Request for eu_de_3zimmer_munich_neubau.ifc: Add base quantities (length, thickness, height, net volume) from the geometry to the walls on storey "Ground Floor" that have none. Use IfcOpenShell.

First a look at what the model holds.

```python
import ifcopenshell
import ifcopenshell.util.element
import ifcopenshell.util.unit

model = ifcopenshell.open("eu_de_3zimmer_munich_neubau.ifc")
print(model.schema)
for unit_type in ("LENGTHUNIT", "AREAUNIT", "VOLUMEUNIT"):
    print(unit_type, ifcopenshell.util.unit.calculate_unit_scale(model, unit_type))
storey = next(s for s in model.by_type("IfcBuildingStorey") if s.Name == "Ground Floor")
walls = [e for e in ifcopenshell.util.element.get_decomposition(storey) if e.is_a("IfcWall")]
for e in sorted(walls, key=lambda e: e.id()):
    print(e.id(), e.is_a(), e.Name, list(ifcopenshell.util.element.get_psets(e, qtos_only=True)), sep=" | ")
```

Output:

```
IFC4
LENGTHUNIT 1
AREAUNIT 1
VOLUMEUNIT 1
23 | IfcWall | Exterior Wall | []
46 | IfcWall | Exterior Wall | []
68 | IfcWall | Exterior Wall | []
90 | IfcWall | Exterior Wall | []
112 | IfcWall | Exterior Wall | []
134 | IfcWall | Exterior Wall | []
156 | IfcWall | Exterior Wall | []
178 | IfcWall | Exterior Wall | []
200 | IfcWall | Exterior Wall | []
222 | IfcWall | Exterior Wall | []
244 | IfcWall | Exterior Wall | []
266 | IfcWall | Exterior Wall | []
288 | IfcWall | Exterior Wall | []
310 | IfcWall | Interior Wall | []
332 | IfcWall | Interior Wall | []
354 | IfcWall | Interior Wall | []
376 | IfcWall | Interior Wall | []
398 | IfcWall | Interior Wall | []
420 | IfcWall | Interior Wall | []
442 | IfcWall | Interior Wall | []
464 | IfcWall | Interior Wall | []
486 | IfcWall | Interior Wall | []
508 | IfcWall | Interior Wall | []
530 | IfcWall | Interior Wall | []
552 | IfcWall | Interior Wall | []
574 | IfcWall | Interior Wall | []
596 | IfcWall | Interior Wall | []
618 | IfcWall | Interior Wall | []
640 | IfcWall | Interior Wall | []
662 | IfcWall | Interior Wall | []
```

```python
import ifcopenshell
import ifcopenshell.api.pset
import ifcopenshell.geom
import ifcopenshell.util.element
import ifcopenshell.util.shape
import ifcopenshell.util.unit

model = ifcopenshell.open("eu_de_3zimmer_munich_neubau.ifc")
unit_scale = ifcopenshell.util.unit.calculate_unit_scale(model)
volume_scale = ifcopenshell.util.unit.calculate_unit_scale(model, "VOLUMEUNIT")
settings = ifcopenshell.geom.settings()

storey = next(s for s in model.by_type("IfcBuildingStorey") if s.Name == "Ground Floor")
walls = [e for e in ifcopenshell.util.element.get_decomposition(storey) if e.is_a("IfcWall")]

for e in sorted(walls, key=lambda e: e.id()):
    if ifcopenshell.util.element.get_psets(e, qtos_only=True, should_inherit=False):
        continue
    # Geometry comes back in metres, in the element's own axes.
    shape = ifcopenshell.geom.create_shape(settings, e)
    values = {
        "Length": ifcopenshell.util.shape.get_x(shape.geometry) / unit_scale,
        "Width": ifcopenshell.util.shape.get_y(shape.geometry) / unit_scale,
        "Height": ifcopenshell.util.shape.get_z(shape.geometry) / unit_scale,
        "NetVolume": ifcopenshell.util.shape.get_volume(shape.geometry) / volume_scale,
    }
    qto = ifcopenshell.api.pset.add_qto(model, product=e, name="Qto_WallBaseQuantities")
    ifcopenshell.api.pset.edit_qto(model, qto=qto, properties=values)
    print(e.id(), {k: round(v, 3) for k, v in values.items()})

model.write("eu_de_3zimmer_munich_neubau-out.ifc")
```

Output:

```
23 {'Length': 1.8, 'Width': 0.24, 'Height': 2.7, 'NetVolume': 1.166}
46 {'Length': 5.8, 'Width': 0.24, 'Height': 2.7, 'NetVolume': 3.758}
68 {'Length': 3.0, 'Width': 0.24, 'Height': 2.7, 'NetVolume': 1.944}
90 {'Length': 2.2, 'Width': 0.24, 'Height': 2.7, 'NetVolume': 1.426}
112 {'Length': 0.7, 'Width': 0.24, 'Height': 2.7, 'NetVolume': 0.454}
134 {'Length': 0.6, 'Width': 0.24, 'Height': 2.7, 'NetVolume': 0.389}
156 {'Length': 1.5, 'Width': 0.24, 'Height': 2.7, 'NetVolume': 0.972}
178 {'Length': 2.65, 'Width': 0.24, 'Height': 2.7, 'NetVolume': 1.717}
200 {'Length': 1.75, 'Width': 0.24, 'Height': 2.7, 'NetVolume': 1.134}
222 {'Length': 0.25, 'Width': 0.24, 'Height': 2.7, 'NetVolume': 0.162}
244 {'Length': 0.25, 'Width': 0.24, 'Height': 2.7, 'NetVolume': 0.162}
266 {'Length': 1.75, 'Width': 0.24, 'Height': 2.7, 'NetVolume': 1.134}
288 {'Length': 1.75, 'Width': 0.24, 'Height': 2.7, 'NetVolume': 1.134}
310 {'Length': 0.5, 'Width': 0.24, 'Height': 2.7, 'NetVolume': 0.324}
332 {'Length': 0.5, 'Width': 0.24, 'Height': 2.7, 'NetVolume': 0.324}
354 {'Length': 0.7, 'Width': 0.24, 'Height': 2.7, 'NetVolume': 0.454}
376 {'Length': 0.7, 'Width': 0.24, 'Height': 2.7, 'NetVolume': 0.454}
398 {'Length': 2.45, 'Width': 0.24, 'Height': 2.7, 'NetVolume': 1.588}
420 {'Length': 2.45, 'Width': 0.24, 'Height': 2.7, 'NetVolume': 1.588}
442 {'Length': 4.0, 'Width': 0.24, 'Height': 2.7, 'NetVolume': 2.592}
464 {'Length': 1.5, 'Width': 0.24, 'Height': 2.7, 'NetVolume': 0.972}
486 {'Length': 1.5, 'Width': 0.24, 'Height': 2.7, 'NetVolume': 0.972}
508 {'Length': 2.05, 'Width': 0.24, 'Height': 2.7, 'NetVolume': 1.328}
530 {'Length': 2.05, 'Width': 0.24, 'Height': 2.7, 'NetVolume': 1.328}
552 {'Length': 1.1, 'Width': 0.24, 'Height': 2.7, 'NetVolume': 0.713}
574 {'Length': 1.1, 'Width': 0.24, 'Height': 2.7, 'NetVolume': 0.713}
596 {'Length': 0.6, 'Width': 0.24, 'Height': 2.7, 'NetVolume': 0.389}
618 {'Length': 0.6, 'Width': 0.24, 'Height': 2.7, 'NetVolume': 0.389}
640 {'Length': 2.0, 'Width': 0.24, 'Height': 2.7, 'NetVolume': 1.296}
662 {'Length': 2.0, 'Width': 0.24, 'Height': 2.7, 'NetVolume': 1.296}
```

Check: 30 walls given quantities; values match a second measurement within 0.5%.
